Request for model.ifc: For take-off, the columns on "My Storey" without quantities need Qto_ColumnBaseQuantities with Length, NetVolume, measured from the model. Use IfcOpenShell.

First a look at what the model holds.

```python
import ifcopenshell
import ifcopenshell.util.element
import ifcopenshell.util.unit

model = ifcopenshell.open("model.ifc")
print(model.schema)
for unit_type in ("LENGTHUNIT", "AREAUNIT", "VOLUMEUNIT"):
    print(unit_type, ifcopenshell.util.unit.calculate_unit_scale(model, unit_type))
storey = next(s for s in model.by_type("IfcBuildingStorey") if s.Name == "My Storey")
columns = [e for e in ifcopenshell.util.element.get_decomposition(storey) if e.is_a("IfcColumn")]
for e in sorted(columns, key=lambda e: e.id()):
    print(e.id(), e.is_a(), e.Name, list(ifcopenshell.util.element.get_psets(e, qtos_only=True)), sep=" | ")
```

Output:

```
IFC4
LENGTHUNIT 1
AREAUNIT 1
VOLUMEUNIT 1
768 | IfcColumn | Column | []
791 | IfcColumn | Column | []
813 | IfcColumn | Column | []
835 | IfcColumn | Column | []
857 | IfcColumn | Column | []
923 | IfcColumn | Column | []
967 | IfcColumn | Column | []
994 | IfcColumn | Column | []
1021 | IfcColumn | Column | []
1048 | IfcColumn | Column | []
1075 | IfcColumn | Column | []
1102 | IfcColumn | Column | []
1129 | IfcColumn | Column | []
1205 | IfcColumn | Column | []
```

```python
import ifcopenshell
import ifcopenshell.api.pset
import ifcopenshell.geom
import ifcopenshell.util.element
import ifcopenshell.util.shape
import ifcopenshell.util.unit

model = ifcopenshell.open("model.ifc")
unit_scale = ifcopenshell.util.unit.calculate_unit_scale(model)
volume_scale = ifcopenshell.util.unit.calculate_unit_scale(model, "VOLUMEUNIT")
settings = ifcopenshell.geom.settings()

storey = next(s for s in model.by_type("IfcBuildingStorey") if s.Name == "My Storey")
columns = [e for e in ifcopenshell.util.element.get_decomposition(storey) if e.is_a("IfcColumn")]

for e in sorted(columns, key=lambda e: e.id()):
    if ifcopenshell.util.element.get_psets(e, qtos_only=True, should_inherit=False):
        continue
    # Geometry comes back in metres, in the element's own axes.
    shape = ifcopenshell.geom.create_shape(settings, e)
    values = {
        "Length": ifcopenshell.util.shape.get_z(shape.geometry) / unit_scale,
        "NetVolume": ifcopenshell.util.shape.get_volume(shape.geometry) / volume_scale,
    }
    qto = ifcopenshell.api.pset.add_qto(model, product=e, name="Qto_ColumnBaseQuantities")
    ifcopenshell.api.pset.edit_qto(model, qto=qto, properties=values)
    print(e.id(), {k: round(v, 3) for k, v in values.items()})

model.write("model-out.ifc")
```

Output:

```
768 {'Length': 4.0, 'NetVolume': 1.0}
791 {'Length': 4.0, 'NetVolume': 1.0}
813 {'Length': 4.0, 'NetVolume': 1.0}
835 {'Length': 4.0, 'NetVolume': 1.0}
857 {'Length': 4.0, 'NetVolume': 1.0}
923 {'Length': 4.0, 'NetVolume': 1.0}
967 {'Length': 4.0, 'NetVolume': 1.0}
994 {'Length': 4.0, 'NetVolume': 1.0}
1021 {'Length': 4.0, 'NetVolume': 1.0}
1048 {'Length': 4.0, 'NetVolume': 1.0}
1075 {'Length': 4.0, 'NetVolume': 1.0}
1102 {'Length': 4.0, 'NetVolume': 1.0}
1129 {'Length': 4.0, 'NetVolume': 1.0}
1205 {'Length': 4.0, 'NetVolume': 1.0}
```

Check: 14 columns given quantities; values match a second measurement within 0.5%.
